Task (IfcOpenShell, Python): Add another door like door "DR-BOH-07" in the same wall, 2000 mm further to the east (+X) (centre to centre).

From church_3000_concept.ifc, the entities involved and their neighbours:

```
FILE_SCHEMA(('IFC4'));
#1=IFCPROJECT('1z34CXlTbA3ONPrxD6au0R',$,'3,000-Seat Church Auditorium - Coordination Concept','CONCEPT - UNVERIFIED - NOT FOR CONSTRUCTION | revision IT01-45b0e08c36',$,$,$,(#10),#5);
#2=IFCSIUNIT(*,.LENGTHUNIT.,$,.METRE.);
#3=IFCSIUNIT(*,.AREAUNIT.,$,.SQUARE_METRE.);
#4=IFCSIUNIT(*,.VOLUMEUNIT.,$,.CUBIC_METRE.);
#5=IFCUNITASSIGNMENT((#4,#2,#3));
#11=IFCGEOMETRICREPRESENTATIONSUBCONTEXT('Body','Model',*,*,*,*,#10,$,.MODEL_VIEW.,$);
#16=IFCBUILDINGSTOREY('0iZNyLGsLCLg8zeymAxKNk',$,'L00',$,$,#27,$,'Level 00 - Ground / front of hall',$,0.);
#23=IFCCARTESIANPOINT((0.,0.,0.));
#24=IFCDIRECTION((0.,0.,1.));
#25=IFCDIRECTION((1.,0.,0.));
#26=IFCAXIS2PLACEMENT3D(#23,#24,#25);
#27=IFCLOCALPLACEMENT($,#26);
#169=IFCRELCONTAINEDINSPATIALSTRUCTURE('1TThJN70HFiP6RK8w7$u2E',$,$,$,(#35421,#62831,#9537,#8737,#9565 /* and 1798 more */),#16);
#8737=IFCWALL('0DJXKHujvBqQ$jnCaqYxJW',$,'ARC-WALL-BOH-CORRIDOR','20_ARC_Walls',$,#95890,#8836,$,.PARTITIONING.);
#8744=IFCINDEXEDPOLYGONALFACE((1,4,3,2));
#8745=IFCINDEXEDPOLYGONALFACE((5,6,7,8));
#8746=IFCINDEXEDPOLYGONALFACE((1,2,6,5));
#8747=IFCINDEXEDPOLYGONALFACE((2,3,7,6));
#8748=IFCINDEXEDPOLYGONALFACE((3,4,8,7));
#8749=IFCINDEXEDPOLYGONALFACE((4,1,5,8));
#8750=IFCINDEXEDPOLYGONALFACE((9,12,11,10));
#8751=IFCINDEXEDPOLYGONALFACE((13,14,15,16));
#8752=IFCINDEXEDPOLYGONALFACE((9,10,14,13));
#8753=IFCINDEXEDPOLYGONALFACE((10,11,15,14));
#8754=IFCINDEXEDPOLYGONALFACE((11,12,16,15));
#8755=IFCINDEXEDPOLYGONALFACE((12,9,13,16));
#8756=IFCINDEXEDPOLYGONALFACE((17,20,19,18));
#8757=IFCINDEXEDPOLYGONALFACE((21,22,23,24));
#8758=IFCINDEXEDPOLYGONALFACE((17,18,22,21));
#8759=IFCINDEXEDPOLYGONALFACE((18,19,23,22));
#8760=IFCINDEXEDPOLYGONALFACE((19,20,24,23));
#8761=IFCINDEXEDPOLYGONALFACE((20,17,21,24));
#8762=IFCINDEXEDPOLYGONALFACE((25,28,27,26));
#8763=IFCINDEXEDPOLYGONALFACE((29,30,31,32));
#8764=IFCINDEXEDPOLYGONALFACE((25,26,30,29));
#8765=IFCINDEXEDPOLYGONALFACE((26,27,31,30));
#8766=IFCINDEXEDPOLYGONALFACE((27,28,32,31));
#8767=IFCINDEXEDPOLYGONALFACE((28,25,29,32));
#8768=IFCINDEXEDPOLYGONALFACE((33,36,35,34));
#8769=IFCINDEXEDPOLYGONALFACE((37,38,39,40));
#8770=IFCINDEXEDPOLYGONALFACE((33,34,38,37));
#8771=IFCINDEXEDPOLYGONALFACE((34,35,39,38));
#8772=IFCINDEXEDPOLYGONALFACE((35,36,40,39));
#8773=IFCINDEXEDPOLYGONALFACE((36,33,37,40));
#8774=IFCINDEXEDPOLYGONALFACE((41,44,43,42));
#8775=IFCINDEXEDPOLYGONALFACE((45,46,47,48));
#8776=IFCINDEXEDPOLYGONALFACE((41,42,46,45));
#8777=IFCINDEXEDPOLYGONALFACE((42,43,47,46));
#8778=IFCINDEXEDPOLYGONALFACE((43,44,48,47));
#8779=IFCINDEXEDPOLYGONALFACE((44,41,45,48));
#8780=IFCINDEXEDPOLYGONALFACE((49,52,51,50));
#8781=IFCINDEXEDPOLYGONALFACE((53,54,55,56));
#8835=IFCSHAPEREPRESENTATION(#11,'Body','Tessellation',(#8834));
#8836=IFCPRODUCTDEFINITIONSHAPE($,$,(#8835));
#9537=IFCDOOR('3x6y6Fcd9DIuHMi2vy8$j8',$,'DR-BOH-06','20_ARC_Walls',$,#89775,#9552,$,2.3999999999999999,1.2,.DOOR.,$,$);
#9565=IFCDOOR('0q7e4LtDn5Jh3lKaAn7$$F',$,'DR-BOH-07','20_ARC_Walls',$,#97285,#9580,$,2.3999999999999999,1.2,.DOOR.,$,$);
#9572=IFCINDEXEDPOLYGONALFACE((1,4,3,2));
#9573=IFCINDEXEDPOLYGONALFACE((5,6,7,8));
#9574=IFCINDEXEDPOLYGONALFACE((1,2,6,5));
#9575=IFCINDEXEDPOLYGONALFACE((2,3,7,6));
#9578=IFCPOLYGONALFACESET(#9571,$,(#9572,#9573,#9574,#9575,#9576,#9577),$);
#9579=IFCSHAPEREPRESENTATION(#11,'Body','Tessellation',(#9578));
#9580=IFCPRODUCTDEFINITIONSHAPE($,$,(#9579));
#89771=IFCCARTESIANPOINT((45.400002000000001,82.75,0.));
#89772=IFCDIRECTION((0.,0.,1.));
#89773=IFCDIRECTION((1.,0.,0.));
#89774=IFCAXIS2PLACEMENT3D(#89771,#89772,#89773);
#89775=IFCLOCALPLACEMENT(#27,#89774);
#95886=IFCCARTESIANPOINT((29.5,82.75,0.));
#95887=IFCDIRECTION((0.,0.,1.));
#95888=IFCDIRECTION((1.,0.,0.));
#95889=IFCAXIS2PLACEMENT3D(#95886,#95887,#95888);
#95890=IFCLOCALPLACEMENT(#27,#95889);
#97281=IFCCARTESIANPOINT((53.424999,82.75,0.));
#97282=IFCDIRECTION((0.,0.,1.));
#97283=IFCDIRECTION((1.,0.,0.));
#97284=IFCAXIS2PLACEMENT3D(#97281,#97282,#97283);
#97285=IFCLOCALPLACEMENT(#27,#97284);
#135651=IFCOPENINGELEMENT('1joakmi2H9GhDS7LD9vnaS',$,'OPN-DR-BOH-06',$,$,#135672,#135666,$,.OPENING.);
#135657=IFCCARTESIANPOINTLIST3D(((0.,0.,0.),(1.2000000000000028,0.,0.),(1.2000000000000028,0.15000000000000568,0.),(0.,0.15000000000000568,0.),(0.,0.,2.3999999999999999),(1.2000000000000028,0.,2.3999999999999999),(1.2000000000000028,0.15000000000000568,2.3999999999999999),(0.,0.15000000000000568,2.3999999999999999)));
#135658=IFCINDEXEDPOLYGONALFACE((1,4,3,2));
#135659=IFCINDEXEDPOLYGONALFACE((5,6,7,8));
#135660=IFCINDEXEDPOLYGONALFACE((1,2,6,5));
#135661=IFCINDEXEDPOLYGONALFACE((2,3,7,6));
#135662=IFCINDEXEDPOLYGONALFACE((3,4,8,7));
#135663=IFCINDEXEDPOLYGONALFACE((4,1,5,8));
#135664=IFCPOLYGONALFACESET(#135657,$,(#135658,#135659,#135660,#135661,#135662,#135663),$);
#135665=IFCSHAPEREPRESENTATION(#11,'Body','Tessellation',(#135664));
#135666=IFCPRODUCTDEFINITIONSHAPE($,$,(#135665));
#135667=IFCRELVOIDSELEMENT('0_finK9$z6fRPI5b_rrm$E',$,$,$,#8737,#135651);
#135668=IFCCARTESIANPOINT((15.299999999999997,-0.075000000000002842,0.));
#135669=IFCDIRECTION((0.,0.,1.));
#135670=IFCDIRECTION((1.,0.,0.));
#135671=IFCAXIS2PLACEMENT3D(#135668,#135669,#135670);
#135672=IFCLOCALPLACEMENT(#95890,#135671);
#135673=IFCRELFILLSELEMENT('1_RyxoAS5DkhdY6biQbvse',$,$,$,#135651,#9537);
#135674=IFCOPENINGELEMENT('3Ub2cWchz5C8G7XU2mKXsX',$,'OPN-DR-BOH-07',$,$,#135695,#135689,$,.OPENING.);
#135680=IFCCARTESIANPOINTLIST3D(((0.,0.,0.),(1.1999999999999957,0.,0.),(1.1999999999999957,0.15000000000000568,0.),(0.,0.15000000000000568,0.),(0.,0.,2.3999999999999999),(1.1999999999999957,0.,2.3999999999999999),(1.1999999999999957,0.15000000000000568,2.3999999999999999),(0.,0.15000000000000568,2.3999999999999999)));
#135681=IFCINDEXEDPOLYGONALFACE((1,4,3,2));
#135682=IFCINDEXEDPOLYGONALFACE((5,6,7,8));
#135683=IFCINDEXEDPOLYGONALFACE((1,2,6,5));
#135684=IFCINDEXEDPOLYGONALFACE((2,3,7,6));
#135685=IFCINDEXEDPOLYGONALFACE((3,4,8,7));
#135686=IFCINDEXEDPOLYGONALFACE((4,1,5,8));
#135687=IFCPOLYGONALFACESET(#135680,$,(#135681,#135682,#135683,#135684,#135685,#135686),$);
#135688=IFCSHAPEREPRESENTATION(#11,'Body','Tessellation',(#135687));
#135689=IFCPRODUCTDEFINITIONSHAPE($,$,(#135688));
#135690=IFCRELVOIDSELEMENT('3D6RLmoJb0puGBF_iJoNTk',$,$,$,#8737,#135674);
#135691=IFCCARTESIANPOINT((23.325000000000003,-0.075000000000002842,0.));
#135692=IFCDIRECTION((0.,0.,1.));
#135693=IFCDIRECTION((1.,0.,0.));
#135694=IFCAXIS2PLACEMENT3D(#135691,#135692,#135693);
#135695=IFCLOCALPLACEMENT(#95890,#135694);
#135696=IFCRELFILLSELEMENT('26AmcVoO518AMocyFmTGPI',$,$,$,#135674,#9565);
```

```python
import ifcopenshell
import ifcopenshell.api.feature
import ifcopenshell.api.geometry
import ifcopenshell.api.root
import ifcopenshell.geom
import ifcopenshell.util.element
import ifcopenshell.util.placement
import ifcopenshell.util.shape
import ifcopenshell.util.unit

model = ifcopenshell.open("church_3000_concept.ifc")
unit_scale = ifcopenshell.util.unit.calculate_unit_scale(model)
settings = ifcopenshell.geom.settings()


def volume(element):
    """Net volume in cubic metres, openings subtracted."""
    shape = ifcopenshell.geom.create_shape(settings, element)
    return ifcopenshell.util.shape.get_volume(shape.geometry)


door = model.by_id(9565)
opening = door.FillsVoids[0].RelatingOpeningElement
wall = opening.VoidsElements[0].RelatingBuildingElement
before = volume(wall)
shift = ifcopenshell.util.placement.get_local_placement(wall.ObjectPlacement)[:3, 0] * 2 / unit_scale

# copy_class copies the void relationship, type, container and properties, but no geometry.
new_opening = ifcopenshell.api.root.copy_class(model, product=opening)
new_opening.Representation = ifcopenshell.util.element.copy_deep(
    model, opening.Representation, exclude=["IfcGeometricRepresentationContext", "IfcRepresentationMap"]
)
new_door = ifcopenshell.api.root.copy_class(model, product=door)
new_door.Representation = ifcopenshell.util.element.copy_deep(
    model, door.Representation, exclude=["IfcGeometricRepresentationContext", "IfcRepresentationMap"]
)
ifcopenshell.api.feature.add_filling(model, opening=new_opening, element=new_door)

for old, new in ((opening, new_opening), (door, new_door)):
    matrix = ifcopenshell.util.placement.get_local_placement(old.ObjectPlacement)
    matrix[:3, 3] += shift
    ifcopenshell.api.geometry.edit_object_placement(model, product=new, matrix=matrix, is_si=False)

after = volume(wall)

print(f"wall volume {before:.3f} -> {after:.3f} m3")

model.write("church_3000_concept_v2.ifc")
```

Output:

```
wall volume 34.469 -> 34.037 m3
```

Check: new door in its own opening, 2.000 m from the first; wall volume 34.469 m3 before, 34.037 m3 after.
